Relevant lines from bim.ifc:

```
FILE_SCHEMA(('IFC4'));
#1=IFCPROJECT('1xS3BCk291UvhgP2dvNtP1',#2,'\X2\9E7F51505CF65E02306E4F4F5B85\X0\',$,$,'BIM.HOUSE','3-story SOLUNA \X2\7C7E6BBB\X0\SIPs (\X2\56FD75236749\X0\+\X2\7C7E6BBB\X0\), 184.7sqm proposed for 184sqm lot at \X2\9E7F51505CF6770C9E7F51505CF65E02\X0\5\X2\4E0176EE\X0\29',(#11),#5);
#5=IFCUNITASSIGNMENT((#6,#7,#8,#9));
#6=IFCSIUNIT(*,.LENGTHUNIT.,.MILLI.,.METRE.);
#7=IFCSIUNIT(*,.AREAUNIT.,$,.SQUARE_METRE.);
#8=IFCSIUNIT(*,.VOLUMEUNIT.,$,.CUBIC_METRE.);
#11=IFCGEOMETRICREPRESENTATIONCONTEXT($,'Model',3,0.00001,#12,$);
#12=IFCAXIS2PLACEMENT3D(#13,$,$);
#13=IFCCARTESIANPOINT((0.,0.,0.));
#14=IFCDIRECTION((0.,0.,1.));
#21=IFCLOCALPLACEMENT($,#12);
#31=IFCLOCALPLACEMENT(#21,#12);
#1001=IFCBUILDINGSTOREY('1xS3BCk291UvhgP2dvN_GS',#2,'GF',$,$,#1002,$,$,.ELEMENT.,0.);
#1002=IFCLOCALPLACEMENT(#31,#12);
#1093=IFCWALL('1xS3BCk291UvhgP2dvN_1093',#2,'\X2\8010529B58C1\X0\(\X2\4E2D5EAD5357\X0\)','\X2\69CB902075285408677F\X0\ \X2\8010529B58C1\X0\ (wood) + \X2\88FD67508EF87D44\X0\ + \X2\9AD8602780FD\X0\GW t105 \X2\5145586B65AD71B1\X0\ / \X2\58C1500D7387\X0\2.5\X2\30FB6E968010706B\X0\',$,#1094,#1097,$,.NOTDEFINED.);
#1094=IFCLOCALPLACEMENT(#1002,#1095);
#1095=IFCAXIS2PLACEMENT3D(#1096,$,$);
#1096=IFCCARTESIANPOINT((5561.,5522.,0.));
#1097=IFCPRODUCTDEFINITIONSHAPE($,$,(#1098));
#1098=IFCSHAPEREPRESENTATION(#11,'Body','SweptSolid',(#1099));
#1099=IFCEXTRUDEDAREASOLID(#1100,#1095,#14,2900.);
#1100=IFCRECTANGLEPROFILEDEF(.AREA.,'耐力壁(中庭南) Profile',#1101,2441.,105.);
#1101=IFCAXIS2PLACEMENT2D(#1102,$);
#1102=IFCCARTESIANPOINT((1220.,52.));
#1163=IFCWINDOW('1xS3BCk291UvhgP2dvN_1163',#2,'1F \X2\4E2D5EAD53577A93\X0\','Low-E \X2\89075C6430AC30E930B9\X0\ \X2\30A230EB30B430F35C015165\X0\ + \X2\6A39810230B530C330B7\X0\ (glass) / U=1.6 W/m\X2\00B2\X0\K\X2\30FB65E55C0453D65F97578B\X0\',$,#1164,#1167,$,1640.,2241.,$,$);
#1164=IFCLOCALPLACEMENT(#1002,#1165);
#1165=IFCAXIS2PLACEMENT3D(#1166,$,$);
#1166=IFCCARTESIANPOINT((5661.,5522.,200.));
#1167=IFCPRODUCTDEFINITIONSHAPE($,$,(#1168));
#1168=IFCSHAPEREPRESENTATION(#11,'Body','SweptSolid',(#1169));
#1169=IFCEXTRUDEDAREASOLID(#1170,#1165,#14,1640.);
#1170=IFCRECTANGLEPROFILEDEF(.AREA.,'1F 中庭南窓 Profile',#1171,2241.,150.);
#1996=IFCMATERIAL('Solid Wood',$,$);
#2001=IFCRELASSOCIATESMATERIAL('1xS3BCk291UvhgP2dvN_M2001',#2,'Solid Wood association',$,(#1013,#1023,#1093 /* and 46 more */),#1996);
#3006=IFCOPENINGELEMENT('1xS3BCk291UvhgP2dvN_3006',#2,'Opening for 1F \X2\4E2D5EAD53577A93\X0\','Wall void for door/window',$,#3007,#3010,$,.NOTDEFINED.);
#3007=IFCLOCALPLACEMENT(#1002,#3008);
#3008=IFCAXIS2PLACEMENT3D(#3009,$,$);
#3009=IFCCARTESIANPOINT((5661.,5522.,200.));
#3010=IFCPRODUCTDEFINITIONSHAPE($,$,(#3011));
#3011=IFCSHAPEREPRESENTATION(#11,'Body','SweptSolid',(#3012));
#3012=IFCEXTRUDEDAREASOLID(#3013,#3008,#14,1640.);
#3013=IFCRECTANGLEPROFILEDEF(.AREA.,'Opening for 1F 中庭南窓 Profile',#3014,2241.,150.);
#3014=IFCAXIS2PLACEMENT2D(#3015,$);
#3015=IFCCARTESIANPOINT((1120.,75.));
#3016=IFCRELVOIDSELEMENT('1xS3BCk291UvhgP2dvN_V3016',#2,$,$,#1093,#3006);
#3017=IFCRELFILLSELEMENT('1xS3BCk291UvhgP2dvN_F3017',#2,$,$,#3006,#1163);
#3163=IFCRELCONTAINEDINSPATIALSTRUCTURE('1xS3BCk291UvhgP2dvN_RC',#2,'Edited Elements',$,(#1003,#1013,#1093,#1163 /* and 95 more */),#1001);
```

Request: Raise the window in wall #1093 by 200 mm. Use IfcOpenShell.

```python
import numpy as np
import ifcopenshell
import ifcopenshell.api.geometry
import ifcopenshell.util.placement
import ifcopenshell.util.unit

model = ifcopenshell.open("bim.ifc")
unit_scale = ifcopenshell.util.unit.calculate_unit_scale(model)

window = model.by_id(1163)
opening = window.FillsVoids[0].RelatingOpeningElement
dz = 0.2 / unit_scale

shift = np.array([0.0, 0.0, dz])
# The window is not placed relative to its opening, so move both.
for product in (opening, window):
    matrix = ifcopenshell.util.placement.get_local_placement(product.ObjectPlacement)
    matrix[:3, 3] += shift
    ifcopenshell.api.geometry.edit_object_placement(model, product=product, matrix=matrix, is_si=False)

print(f"moved by {dz * unit_scale:+.3f} m")

model.write("bim-out.ifc")
```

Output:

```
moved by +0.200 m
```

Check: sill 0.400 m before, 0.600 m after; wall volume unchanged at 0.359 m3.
